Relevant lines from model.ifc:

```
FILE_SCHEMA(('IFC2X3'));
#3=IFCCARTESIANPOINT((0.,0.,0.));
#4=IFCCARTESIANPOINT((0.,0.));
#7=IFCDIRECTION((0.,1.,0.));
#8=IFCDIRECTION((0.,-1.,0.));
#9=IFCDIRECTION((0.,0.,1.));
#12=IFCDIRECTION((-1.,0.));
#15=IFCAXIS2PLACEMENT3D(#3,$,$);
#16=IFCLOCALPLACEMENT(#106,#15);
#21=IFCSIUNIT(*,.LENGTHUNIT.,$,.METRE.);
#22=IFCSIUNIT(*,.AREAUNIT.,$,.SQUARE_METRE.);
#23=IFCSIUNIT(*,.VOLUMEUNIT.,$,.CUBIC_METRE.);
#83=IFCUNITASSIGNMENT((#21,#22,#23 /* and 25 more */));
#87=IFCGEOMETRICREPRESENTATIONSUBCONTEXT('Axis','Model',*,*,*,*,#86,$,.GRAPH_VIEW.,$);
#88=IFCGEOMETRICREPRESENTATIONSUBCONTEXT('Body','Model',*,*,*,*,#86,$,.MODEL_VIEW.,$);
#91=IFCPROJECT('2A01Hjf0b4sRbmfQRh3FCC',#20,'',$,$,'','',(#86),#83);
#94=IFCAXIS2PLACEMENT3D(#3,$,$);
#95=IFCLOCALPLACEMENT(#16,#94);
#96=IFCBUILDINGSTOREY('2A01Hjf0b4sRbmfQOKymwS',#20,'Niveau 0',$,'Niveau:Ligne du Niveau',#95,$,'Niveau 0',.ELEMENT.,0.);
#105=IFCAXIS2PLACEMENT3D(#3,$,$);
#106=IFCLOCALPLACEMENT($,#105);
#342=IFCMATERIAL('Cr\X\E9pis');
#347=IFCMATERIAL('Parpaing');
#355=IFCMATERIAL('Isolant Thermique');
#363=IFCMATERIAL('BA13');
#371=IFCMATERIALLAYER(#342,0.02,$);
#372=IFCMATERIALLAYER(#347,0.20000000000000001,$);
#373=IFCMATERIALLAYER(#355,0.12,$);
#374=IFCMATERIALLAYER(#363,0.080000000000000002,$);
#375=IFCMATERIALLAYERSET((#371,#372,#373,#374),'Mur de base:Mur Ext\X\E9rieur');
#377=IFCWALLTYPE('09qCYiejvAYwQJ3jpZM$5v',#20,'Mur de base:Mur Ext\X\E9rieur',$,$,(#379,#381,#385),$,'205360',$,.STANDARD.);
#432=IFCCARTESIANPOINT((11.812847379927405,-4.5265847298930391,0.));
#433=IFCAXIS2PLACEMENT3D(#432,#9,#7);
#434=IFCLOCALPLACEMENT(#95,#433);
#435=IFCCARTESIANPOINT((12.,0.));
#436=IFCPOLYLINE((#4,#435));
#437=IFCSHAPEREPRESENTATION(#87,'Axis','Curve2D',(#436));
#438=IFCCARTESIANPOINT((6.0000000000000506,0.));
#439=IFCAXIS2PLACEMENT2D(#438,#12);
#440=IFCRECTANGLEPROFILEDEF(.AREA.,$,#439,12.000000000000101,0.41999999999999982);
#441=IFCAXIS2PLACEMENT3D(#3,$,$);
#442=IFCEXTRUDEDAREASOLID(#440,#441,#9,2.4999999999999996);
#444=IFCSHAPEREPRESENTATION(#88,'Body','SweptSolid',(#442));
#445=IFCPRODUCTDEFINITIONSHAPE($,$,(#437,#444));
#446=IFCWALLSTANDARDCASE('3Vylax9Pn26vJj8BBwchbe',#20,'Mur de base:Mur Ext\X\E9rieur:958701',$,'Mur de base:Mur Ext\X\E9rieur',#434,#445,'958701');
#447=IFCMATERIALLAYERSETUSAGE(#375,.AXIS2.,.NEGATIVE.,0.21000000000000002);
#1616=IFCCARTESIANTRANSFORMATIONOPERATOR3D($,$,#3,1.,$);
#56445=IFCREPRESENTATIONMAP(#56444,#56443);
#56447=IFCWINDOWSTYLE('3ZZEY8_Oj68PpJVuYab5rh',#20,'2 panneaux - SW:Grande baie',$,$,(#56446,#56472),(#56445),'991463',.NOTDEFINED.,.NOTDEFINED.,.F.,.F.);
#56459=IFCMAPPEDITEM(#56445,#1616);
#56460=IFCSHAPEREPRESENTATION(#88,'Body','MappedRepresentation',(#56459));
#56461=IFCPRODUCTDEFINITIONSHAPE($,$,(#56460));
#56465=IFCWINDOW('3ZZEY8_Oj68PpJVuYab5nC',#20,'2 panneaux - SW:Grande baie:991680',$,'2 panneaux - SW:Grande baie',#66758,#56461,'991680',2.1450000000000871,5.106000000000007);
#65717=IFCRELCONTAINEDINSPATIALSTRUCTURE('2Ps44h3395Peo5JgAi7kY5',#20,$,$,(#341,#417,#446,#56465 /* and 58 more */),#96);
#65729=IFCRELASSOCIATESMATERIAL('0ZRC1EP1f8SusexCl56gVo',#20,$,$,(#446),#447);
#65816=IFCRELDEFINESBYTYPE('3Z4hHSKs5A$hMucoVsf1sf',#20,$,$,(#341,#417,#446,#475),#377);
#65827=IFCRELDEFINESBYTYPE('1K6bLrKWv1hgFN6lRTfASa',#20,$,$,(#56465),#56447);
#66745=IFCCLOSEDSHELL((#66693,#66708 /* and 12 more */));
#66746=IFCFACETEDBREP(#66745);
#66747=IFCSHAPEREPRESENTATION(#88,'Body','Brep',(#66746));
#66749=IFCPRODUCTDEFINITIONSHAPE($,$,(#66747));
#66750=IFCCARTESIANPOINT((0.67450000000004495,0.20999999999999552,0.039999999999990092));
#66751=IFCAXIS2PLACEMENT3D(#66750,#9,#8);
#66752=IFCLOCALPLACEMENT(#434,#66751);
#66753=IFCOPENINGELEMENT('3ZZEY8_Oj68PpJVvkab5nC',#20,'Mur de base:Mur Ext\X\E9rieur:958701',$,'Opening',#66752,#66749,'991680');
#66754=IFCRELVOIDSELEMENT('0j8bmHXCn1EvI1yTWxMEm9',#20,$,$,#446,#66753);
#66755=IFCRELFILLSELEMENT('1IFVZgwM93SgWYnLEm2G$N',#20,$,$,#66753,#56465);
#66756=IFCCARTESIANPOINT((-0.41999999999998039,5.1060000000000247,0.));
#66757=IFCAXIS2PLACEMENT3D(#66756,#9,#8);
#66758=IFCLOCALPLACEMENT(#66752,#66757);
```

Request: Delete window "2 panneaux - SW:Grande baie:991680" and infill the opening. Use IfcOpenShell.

```python
import ifcopenshell
import ifcopenshell.api.feature
import ifcopenshell.api.root
import ifcopenshell.geom
import ifcopenshell.util.shape

model = ifcopenshell.open("model.ifc")
settings = ifcopenshell.geom.settings()


def volume(element):
    """Net volume in cubic metres, openings subtracted."""
    shape = ifcopenshell.geom.create_shape(settings, element)
    return ifcopenshell.util.shape.get_volume(shape.geometry)


window = model.by_guid("3ZZEY8_Oj68PpJVuYab5nC")
opening = window.FillsVoids[0].RelatingOpeningElement
wall = opening.VoidsElements[0].RelatingBuildingElement
before = volume(wall)

ifcopenshell.api.root.remove_product(model, product=window)
ifcopenshell.api.feature.remove_feature(model, feature=opening)

after = volume(wall)

print(f"wall volume {before:.3f} -> {after:.3f} m3")

model.write("model-out.ifc")
```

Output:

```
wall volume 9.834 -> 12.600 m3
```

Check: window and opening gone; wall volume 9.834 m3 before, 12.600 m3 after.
